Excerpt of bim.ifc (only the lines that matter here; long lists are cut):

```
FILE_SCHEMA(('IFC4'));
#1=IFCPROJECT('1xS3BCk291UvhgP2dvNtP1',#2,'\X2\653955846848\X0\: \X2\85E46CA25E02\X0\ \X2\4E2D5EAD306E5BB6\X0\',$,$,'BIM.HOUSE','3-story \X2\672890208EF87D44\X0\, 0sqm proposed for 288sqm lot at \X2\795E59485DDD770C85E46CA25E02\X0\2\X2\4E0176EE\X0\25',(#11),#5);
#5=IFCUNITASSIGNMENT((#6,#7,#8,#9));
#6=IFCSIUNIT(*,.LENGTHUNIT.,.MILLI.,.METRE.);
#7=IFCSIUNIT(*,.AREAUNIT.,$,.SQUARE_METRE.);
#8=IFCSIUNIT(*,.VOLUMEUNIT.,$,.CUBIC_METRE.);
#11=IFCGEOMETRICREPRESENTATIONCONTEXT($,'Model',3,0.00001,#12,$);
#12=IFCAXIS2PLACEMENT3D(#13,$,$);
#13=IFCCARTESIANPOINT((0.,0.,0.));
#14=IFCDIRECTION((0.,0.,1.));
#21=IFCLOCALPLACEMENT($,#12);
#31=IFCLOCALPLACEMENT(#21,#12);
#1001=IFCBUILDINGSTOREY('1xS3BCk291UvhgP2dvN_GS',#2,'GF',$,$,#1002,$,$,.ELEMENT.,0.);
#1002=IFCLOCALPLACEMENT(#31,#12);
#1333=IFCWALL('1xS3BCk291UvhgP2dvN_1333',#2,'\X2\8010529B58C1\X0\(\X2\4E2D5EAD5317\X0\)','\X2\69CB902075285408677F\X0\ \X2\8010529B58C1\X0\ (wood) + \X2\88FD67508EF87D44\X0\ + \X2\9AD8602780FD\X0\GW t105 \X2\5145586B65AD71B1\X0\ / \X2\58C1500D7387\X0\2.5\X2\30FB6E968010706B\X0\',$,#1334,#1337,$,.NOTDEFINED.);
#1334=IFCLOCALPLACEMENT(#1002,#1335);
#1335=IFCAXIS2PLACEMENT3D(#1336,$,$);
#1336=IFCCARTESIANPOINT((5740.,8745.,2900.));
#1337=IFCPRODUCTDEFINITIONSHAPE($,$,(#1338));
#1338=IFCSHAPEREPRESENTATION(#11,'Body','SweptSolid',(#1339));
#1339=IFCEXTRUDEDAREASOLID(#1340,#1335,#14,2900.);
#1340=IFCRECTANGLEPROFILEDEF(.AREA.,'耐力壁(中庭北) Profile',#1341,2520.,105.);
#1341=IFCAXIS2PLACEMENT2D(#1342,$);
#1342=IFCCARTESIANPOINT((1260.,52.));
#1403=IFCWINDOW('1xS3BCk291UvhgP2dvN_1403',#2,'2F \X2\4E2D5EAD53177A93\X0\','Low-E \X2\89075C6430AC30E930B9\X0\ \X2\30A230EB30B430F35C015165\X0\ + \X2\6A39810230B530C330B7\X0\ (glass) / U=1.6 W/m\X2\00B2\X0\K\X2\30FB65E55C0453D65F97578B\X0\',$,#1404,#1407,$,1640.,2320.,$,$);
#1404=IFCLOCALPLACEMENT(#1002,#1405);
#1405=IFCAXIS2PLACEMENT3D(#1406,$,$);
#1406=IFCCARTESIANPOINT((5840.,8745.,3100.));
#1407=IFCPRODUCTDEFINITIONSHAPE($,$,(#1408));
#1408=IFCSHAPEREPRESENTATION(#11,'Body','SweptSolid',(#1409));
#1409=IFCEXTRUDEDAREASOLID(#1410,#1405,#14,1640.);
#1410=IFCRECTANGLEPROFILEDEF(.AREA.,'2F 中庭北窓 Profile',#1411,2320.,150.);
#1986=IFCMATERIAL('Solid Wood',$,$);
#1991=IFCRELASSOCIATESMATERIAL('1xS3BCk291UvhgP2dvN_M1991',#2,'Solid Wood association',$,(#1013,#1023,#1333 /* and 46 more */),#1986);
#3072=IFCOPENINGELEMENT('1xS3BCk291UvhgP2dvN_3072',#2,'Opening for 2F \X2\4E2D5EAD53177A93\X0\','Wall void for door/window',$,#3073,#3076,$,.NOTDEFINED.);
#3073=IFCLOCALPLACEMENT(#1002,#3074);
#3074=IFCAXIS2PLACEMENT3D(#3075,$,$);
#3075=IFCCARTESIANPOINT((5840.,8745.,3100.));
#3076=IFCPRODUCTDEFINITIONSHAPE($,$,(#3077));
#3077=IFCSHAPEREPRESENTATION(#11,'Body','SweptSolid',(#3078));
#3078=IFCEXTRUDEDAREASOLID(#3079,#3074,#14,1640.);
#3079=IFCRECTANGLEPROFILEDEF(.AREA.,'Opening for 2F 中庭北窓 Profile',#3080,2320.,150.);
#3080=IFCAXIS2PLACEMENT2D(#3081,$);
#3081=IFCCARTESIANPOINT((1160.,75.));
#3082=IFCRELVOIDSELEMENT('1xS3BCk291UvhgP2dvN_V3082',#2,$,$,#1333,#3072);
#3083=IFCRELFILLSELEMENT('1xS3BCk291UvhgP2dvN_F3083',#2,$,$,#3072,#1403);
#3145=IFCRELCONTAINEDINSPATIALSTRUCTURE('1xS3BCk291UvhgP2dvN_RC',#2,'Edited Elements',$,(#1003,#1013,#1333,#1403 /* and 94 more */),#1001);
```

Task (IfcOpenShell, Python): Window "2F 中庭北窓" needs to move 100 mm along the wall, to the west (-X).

```python
import ifcopenshell
import ifcopenshell.api.geometry
import ifcopenshell.util.placement

model = ifcopenshell.open("bim.ifc")

window = model.by_guid("1xS3BCk291UvhgP2dvN_1403")
opening = window.FillsVoids[0].RelatingOpeningElement
wall = opening.VoidsElements[0].RelatingBuildingElement

wall_matrix = ifcopenshell.util.placement.get_local_placement(wall.ObjectPlacement)
shift = wall_matrix[:3, 0] * -100.0
before = ifcopenshell.util.placement.get_local_placement(window.ObjectPlacement)[:3, 3].copy()

# The window is not placed relative to its opening, so move both.
for product in (opening, window):
    matrix = ifcopenshell.util.placement.get_local_placement(product.ObjectPlacement)
    matrix[:3, 3] += shift
    ifcopenshell.api.geometry.edit_object_placement(model, product=product, matrix=matrix, is_si=False)

after = ifcopenshell.util.placement.get_local_placement(window.ObjectPlacement)[:3, 3]
print("window moved by", (after - before).round(3) + 0.0)

model.write("bim_edited.ifc")
```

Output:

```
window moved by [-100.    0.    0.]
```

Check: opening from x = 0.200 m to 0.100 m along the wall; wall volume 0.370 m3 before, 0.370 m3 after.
